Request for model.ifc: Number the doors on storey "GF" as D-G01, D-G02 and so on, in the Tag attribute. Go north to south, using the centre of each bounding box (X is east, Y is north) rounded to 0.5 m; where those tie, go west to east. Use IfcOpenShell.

First a look at what the model holds.

```python
import ifcopenshell
import ifcopenshell.util.element
import ifcopenshell.util.placement

model = ifcopenshell.open("model.ifc")
print(model.schema)
storey = next(s for s in model.by_type("IfcBuildingStorey") if s.Name == "GF")
doors = [e for e in ifcopenshell.util.element.get_decomposition(storey) if e.is_a("IfcDoor")]
for e in sorted(doors, key=lambda e: e.id()):
    origin = ifcopenshell.util.placement.get_local_placement(e.ObjectPlacement)[:3, 3]
    print(e.id(), e.Tag, e.Name, origin.round(2) + 0.0, sep=" | ")
```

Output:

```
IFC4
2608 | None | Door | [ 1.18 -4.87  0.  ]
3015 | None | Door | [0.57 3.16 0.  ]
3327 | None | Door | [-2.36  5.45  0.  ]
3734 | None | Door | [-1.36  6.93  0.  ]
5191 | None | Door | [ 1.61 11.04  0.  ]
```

```python
import ifcopenshell
import ifcopenshell.geom
import ifcopenshell.util.element
import ifcopenshell.util.shape

model = ifcopenshell.open("model.ifc")
settings = ifcopenshell.geom.settings()
settings.set("use-world-coords", True)


def centre(element):
    shape = ifcopenshell.geom.create_shape(settings, element)
    return ifcopenshell.util.shape.get_bbox_centroid(shape.geometry)


storey = next(s for s in model.by_type("IfcBuildingStorey") if s.Name == "GF")
doors = [e for e in ifcopenshell.util.element.get_decomposition(storey) if e.is_a("IfcDoor")]

# Insertion points can sit at a corner or the storey origin, so sort by the geometry (in metres).
centres = {e: centre(e) for e in doors}
doors.sort(key=lambda e: (-round(centres[e][1] / 0.5), centres[e][0]))

for i, e in enumerate(doors, start=1):
    number = f"D-G{i:02d}"
    e.Tag = number
    print(e.id(), number)

model.write("model-out.ifc")
```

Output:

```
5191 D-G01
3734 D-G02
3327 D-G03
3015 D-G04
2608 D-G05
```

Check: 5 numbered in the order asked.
